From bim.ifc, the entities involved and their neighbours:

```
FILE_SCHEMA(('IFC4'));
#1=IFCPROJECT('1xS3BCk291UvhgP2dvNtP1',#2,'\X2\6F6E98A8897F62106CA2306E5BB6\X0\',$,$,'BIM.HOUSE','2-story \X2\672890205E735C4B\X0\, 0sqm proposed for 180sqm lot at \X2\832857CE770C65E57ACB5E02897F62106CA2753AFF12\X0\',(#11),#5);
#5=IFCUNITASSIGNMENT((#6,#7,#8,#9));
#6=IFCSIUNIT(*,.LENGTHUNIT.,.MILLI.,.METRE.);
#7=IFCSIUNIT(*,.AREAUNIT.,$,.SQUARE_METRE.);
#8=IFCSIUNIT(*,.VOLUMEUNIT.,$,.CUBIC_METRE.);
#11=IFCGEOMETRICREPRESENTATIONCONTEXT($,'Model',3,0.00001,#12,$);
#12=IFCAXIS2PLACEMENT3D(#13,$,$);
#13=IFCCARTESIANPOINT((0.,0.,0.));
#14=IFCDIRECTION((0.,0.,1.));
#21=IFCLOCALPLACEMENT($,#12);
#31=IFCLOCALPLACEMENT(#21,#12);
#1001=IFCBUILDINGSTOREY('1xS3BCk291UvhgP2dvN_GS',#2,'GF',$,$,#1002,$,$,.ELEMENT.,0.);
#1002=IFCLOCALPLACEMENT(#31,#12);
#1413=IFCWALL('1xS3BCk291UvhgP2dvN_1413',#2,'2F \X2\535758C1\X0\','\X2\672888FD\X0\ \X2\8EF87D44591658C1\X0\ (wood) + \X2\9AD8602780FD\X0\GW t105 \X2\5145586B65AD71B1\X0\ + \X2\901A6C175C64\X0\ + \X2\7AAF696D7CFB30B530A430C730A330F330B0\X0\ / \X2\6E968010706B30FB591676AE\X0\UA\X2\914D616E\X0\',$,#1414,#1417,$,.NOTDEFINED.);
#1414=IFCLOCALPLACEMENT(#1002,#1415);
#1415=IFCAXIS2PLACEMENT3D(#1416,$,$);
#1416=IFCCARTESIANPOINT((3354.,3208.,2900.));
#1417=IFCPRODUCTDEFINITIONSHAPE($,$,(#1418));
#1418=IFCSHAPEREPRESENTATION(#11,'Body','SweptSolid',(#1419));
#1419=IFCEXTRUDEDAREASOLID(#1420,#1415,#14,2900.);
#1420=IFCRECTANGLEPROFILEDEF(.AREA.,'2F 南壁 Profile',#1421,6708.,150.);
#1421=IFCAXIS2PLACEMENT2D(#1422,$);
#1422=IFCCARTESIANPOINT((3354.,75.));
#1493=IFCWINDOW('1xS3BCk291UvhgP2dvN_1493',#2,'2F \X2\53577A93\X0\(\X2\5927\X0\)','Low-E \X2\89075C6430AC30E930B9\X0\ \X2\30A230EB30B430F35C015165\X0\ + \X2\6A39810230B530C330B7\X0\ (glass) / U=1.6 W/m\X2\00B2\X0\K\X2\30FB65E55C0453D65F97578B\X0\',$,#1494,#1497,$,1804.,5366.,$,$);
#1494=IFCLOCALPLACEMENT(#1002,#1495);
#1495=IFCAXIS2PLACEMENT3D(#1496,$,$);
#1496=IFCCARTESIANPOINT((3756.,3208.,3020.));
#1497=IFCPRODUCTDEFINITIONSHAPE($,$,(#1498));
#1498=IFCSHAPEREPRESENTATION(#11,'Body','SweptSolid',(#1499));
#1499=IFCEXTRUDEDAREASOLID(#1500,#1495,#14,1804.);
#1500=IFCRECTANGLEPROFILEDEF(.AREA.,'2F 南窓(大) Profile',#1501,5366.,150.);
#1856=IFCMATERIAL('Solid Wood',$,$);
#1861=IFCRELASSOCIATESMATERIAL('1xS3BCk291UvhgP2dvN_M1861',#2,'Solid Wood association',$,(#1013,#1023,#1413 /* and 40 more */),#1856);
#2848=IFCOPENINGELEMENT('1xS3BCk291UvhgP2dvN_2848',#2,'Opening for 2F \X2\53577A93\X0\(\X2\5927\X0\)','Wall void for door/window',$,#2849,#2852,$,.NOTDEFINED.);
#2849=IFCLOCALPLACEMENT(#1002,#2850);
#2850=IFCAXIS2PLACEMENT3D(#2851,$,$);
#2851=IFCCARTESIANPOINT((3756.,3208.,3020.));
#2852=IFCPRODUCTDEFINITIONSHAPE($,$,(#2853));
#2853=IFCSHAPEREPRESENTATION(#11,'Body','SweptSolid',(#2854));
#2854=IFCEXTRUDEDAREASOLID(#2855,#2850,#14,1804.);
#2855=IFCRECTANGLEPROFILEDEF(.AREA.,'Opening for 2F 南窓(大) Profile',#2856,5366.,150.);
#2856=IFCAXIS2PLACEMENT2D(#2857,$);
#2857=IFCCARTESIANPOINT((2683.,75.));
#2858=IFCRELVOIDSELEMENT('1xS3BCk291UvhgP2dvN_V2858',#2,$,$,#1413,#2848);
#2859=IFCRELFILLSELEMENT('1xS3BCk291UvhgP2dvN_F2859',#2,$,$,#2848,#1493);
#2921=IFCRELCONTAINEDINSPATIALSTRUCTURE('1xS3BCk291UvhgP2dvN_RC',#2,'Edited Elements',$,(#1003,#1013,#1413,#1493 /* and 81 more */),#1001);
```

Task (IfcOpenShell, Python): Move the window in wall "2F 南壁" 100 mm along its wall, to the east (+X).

```python
import ifcopenshell
import ifcopenshell.api.geometry
import ifcopenshell.util.placement

model = ifcopenshell.open("bim.ifc")

window = model.by_guid("1xS3BCk291UvhgP2dvN_1493")
opening = window.FillsVoids[0].RelatingOpeningElement
wall = opening.VoidsElements[0].RelatingBuildingElement

wall_matrix = ifcopenshell.util.placement.get_local_placement(wall.ObjectPlacement)
shift = wall_matrix[:3, 0] * 100.0
before = ifcopenshell.util.placement.get_local_placement(window.ObjectPlacement)[:3, 3].copy()

# The window is not placed relative to its opening, so move both.
for product in (opening, window):
    matrix = ifcopenshell.util.placement.get_local_placement(product.ObjectPlacement)
    matrix[:3, 3] += shift
    ifcopenshell.api.geometry.edit_object_placement(model, product=product, matrix=matrix, is_si=False)

after = ifcopenshell.util.placement.get_local_placement(window.ObjectPlacement)[:3, 3]
print("window moved by", (after - before).round(3) + 0.0)

model.write("bim_v2.ifc")
```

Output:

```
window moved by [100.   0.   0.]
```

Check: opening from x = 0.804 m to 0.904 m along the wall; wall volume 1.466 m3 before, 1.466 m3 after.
